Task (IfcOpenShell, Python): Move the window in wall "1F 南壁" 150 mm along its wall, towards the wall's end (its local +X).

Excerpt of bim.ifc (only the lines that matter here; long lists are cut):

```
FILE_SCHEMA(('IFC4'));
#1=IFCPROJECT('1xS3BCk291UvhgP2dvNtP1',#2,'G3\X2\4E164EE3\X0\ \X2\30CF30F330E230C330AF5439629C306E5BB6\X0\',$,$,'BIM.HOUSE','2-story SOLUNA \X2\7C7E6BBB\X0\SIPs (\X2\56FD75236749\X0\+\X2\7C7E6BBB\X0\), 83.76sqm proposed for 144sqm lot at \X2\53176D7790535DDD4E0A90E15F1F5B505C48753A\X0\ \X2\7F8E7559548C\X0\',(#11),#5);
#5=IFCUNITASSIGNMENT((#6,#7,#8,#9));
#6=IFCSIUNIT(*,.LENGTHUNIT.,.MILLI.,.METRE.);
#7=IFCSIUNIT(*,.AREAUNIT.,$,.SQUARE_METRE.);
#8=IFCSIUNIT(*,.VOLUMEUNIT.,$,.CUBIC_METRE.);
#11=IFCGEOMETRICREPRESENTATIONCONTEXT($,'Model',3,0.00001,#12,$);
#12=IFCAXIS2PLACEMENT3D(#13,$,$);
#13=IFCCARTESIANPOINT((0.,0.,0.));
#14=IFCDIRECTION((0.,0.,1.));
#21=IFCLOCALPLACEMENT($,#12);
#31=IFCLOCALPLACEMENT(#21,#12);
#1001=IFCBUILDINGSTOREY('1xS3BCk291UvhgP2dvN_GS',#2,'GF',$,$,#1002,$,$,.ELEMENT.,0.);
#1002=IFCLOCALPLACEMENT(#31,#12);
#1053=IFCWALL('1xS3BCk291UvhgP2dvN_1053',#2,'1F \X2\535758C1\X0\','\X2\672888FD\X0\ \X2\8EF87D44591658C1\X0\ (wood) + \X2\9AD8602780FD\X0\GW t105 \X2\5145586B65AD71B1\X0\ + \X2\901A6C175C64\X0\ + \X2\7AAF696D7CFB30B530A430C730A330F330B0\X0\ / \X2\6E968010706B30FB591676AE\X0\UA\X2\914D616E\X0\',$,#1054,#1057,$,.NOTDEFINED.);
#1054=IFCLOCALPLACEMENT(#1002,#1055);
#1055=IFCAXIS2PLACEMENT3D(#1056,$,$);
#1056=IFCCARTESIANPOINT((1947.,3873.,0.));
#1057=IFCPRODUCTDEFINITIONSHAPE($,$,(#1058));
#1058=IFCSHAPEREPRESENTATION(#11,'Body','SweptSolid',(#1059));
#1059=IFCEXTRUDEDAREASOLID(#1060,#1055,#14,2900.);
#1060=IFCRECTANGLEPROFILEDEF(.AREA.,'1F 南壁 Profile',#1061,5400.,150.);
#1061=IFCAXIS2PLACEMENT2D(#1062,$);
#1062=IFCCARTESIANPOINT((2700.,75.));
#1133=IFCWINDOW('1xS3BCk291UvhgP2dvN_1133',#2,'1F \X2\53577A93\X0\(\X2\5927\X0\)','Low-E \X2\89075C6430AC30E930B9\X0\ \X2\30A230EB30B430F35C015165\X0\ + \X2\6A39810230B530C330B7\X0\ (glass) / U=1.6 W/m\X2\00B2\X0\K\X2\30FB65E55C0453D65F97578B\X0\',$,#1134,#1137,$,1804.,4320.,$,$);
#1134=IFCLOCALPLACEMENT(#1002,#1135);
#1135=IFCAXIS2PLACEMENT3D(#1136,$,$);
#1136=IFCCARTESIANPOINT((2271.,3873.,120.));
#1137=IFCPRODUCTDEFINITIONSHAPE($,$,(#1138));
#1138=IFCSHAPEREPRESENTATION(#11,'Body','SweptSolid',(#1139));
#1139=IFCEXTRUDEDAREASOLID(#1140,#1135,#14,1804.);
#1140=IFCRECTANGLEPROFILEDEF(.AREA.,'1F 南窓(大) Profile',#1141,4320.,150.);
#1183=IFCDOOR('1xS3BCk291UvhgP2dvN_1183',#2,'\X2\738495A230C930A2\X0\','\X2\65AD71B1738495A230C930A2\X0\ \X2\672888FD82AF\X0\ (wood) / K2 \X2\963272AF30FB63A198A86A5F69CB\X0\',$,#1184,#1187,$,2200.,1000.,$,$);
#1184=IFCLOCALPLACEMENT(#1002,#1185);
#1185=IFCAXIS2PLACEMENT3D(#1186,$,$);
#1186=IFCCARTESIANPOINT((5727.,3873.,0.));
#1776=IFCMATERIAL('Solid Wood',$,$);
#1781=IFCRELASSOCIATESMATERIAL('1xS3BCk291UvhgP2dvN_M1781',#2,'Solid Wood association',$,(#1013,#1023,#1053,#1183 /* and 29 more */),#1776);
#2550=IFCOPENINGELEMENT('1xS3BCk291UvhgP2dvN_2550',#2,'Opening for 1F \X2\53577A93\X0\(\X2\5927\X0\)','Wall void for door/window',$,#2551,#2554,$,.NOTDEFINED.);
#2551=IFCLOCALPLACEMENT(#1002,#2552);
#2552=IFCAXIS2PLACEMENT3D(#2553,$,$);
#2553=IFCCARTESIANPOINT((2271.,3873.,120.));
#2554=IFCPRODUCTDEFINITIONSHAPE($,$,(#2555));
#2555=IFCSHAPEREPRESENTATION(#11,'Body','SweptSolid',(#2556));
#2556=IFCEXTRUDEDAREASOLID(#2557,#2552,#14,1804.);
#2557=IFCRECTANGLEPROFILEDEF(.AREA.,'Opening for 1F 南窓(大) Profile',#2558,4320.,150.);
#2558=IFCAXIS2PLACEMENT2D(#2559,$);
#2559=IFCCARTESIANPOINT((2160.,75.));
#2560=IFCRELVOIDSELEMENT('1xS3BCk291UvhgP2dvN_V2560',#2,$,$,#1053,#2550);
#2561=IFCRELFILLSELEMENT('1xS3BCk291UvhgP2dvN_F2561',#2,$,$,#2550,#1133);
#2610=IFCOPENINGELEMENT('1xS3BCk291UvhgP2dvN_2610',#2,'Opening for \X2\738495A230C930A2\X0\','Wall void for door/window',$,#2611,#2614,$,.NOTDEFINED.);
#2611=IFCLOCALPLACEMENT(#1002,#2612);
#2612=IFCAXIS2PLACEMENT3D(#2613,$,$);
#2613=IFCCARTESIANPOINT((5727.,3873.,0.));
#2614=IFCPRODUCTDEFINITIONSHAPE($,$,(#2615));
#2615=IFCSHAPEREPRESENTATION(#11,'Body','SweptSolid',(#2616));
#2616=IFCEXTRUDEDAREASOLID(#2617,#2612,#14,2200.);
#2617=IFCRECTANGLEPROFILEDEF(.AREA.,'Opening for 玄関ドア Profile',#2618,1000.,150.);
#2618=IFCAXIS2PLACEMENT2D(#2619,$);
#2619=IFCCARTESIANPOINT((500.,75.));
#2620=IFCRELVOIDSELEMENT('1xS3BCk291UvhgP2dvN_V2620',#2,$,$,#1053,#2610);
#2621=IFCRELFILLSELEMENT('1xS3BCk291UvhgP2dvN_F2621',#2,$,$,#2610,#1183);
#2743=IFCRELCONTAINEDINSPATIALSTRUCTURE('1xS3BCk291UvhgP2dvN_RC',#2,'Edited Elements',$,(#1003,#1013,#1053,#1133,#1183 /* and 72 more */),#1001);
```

```python
import ifcopenshell
import ifcopenshell.api.geometry
import ifcopenshell.util.placement
import ifcopenshell.util.unit

model = ifcopenshell.open("bim.ifc")
unit_scale = ifcopenshell.util.unit.calculate_unit_scale(model)

window = model.by_guid("1xS3BCk291UvhgP2dvN_1133")
opening = window.FillsVoids[0].RelatingOpeningElement
wall = opening.VoidsElements[0].RelatingBuildingElement

wall_matrix = ifcopenshell.util.placement.get_local_placement(wall.ObjectPlacement)
shift = wall_matrix[:3, 0] * 0.15 / unit_scale
before = ifcopenshell.util.placement.get_local_placement(window.ObjectPlacement)[:3, 3].copy()

# The window is not placed relative to its opening, so move both.
for product in (opening, window):
    matrix = ifcopenshell.util.placement.get_local_placement(product.ObjectPlacement)
    matrix[:3, 3] += shift
    ifcopenshell.api.geometry.edit_object_placement(model, product=product, matrix=matrix, is_si=False)

after = ifcopenshell.util.placement.get_local_placement(window.ObjectPlacement)[:3, 3]
print("window moved by", (after - before).round(3) + 0.0)

model.write("bim-out.ifc")
```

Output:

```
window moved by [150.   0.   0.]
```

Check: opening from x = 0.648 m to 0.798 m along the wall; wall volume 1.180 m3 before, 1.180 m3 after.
